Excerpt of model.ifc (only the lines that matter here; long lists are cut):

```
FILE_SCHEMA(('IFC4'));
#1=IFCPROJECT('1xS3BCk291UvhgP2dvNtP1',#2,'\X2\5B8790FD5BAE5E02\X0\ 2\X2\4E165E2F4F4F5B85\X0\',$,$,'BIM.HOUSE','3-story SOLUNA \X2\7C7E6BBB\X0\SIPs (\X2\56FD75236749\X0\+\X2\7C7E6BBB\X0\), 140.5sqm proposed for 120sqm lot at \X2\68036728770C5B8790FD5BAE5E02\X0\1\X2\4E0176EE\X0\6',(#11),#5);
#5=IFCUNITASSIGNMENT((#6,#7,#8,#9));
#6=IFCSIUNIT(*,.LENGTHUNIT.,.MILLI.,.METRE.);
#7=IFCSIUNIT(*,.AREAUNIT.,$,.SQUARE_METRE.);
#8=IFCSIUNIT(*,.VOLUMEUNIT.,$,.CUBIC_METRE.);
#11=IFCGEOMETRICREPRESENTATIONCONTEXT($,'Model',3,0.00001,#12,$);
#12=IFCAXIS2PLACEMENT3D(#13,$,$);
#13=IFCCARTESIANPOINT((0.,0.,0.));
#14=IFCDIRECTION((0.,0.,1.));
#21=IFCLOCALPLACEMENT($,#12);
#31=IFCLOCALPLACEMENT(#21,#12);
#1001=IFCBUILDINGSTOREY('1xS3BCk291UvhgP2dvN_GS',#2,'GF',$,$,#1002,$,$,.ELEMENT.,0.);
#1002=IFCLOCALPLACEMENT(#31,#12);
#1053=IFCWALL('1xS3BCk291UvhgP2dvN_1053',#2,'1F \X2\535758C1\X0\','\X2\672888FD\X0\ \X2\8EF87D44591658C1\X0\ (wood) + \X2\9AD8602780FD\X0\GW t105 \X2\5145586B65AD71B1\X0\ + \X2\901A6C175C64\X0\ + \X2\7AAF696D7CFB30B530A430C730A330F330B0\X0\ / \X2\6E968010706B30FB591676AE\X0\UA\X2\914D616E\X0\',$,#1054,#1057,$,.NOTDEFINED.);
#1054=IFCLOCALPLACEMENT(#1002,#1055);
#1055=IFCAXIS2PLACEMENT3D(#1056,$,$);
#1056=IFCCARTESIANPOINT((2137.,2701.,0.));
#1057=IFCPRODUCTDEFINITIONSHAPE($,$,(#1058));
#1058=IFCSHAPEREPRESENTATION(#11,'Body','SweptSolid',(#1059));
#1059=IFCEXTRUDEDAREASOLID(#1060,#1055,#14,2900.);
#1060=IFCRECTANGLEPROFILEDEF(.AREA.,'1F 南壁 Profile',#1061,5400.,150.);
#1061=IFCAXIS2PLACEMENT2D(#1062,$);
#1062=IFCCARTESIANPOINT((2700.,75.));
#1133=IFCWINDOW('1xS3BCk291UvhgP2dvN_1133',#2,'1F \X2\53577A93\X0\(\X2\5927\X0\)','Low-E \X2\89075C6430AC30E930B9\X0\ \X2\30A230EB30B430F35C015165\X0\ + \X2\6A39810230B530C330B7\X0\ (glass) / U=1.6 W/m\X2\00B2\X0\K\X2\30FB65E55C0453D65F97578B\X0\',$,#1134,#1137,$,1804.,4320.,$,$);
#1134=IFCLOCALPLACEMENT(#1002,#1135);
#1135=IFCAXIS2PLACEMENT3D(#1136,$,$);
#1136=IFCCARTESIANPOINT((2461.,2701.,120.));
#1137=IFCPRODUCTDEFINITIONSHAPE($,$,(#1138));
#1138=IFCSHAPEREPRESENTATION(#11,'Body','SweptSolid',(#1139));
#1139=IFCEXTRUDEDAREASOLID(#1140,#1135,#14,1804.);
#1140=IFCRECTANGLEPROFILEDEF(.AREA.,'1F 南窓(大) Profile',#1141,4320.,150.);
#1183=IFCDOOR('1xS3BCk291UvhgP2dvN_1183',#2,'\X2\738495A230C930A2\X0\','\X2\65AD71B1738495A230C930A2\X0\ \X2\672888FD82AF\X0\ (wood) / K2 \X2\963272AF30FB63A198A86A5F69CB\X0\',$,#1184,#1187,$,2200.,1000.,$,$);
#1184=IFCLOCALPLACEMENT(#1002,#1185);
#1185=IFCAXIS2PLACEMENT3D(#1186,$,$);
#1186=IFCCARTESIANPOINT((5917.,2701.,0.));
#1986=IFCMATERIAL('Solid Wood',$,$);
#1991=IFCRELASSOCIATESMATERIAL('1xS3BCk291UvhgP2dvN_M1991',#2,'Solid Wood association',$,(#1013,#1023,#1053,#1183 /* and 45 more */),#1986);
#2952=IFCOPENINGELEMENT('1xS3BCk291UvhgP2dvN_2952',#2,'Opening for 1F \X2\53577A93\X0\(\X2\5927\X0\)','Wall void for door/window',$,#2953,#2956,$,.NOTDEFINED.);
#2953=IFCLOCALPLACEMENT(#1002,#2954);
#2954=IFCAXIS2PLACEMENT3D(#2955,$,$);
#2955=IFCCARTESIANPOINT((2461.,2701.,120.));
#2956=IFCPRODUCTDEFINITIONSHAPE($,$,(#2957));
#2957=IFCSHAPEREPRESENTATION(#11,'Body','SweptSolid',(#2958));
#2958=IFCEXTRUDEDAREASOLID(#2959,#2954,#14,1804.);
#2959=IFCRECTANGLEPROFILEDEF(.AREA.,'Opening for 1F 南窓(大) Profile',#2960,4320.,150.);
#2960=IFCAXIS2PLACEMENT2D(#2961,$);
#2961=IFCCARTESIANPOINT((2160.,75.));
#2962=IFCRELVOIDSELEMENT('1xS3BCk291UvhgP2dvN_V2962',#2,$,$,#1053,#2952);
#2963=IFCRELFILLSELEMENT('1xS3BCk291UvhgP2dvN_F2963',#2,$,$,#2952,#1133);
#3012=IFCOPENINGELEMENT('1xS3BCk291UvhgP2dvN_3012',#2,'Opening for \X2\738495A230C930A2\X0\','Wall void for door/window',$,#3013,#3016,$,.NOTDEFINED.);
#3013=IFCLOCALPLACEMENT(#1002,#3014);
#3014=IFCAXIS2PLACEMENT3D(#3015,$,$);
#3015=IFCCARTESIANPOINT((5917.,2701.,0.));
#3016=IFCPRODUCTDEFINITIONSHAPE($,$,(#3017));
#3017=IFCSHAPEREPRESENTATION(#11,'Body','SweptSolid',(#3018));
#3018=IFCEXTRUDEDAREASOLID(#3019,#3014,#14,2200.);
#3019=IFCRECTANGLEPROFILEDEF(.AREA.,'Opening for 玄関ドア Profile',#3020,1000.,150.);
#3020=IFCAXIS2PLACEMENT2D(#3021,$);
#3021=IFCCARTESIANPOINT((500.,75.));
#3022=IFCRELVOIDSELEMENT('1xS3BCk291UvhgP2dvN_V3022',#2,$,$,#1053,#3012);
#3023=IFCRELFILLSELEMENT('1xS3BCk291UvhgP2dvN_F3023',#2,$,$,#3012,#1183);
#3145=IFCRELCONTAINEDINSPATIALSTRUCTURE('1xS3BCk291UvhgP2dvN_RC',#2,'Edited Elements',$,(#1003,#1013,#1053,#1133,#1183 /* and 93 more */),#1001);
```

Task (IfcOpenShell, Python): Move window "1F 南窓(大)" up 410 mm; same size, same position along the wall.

```python
import numpy as np
import ifcopenshell
import ifcopenshell.api.geometry
import ifcopenshell.util.placement
import ifcopenshell.util.unit

model = ifcopenshell.open("model.ifc")
unit_scale = ifcopenshell.util.unit.calculate_unit_scale(model)

window = model.by_guid("1xS3BCk291UvhgP2dvN_1133")
opening = window.FillsVoids[0].RelatingOpeningElement
dz = 410.0

shift = np.array([0.0, 0.0, dz])
# The window is not placed relative to its opening, so move both.
for product in (opening, window):
    matrix = ifcopenshell.util.placement.get_local_placement(product.ObjectPlacement)
    matrix[:3, 3] += shift
    ifcopenshell.api.geometry.edit_object_placement(model, product=product, matrix=matrix, is_si=False)

print(f"moved by {dz * unit_scale:+.3f} m")

model.write("model_edited.ifc")
```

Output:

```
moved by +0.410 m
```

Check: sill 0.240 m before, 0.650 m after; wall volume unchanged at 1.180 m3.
